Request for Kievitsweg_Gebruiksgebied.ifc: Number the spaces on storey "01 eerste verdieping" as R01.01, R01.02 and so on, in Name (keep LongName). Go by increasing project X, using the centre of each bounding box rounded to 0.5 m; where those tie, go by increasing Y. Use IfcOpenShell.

First a look at what the model holds.

```python
import ifcopenshell
import ifcopenshell.util.element
import ifcopenshell.util.placement

model = ifcopenshell.open("Kievitsweg_Gebruiksgebied.ifc")
print(model.schema)
storey = next(s for s in model.by_type("IfcBuildingStorey") if s.Name == "01 eerste verdieping")
spaces = [e for e in ifcopenshell.util.element.get_decomposition(storey) if e.is_a("IfcSpace")]
for e in sorted(spaces, key=lambda e: e.id()):
    origin = ifcopenshell.util.placement.get_local_placement(e.ObjectPlacement)[:3, 3]
    print(e.id(), e.Name, e.LongName, origin.round(2) + 0.0, sep=" | ")
```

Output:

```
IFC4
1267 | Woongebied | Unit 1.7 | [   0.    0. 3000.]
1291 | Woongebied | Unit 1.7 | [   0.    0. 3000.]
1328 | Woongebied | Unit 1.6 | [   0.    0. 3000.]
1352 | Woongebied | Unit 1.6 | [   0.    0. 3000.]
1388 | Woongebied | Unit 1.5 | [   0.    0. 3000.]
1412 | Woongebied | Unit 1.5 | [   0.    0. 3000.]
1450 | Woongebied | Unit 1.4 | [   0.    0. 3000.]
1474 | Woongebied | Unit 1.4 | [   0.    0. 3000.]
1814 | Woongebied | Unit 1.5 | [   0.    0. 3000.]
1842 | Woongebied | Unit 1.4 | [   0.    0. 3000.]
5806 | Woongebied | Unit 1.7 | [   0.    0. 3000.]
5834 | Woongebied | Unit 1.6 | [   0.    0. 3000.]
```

```python
import ifcopenshell
import ifcopenshell.geom
import ifcopenshell.util.element
import ifcopenshell.util.shape

model = ifcopenshell.open("Kievitsweg_Gebruiksgebied.ifc")
settings = ifcopenshell.geom.settings()
settings.set("use-world-coords", True)


def centre(element):
    shape = ifcopenshell.geom.create_shape(settings, element)
    return ifcopenshell.util.shape.get_bbox_centroid(shape.geometry)


storey = next(s for s in model.by_type("IfcBuildingStorey") if s.Name == "01 eerste verdieping")
spaces = [e for e in ifcopenshell.util.element.get_decomposition(storey) if e.is_a("IfcSpace")]

# Insertion points can sit at a corner or the storey origin, so sort by the geometry (in metres).
centres = {e: centre(e) for e in spaces}
spaces.sort(key=lambda e: (round(centres[e][0] / 0.5), centres[e][1]))

for i, e in enumerate(spaces, start=1):
    number = f"R01.{i:02d}"
    e.Name = number
    print(e.id(), number)

model.write("Kievitsweg_Gebruiksgebied_rev.ifc")
```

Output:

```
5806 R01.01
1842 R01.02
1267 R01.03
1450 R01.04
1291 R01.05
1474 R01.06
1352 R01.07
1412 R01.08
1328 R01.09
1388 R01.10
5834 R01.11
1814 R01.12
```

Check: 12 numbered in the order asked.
